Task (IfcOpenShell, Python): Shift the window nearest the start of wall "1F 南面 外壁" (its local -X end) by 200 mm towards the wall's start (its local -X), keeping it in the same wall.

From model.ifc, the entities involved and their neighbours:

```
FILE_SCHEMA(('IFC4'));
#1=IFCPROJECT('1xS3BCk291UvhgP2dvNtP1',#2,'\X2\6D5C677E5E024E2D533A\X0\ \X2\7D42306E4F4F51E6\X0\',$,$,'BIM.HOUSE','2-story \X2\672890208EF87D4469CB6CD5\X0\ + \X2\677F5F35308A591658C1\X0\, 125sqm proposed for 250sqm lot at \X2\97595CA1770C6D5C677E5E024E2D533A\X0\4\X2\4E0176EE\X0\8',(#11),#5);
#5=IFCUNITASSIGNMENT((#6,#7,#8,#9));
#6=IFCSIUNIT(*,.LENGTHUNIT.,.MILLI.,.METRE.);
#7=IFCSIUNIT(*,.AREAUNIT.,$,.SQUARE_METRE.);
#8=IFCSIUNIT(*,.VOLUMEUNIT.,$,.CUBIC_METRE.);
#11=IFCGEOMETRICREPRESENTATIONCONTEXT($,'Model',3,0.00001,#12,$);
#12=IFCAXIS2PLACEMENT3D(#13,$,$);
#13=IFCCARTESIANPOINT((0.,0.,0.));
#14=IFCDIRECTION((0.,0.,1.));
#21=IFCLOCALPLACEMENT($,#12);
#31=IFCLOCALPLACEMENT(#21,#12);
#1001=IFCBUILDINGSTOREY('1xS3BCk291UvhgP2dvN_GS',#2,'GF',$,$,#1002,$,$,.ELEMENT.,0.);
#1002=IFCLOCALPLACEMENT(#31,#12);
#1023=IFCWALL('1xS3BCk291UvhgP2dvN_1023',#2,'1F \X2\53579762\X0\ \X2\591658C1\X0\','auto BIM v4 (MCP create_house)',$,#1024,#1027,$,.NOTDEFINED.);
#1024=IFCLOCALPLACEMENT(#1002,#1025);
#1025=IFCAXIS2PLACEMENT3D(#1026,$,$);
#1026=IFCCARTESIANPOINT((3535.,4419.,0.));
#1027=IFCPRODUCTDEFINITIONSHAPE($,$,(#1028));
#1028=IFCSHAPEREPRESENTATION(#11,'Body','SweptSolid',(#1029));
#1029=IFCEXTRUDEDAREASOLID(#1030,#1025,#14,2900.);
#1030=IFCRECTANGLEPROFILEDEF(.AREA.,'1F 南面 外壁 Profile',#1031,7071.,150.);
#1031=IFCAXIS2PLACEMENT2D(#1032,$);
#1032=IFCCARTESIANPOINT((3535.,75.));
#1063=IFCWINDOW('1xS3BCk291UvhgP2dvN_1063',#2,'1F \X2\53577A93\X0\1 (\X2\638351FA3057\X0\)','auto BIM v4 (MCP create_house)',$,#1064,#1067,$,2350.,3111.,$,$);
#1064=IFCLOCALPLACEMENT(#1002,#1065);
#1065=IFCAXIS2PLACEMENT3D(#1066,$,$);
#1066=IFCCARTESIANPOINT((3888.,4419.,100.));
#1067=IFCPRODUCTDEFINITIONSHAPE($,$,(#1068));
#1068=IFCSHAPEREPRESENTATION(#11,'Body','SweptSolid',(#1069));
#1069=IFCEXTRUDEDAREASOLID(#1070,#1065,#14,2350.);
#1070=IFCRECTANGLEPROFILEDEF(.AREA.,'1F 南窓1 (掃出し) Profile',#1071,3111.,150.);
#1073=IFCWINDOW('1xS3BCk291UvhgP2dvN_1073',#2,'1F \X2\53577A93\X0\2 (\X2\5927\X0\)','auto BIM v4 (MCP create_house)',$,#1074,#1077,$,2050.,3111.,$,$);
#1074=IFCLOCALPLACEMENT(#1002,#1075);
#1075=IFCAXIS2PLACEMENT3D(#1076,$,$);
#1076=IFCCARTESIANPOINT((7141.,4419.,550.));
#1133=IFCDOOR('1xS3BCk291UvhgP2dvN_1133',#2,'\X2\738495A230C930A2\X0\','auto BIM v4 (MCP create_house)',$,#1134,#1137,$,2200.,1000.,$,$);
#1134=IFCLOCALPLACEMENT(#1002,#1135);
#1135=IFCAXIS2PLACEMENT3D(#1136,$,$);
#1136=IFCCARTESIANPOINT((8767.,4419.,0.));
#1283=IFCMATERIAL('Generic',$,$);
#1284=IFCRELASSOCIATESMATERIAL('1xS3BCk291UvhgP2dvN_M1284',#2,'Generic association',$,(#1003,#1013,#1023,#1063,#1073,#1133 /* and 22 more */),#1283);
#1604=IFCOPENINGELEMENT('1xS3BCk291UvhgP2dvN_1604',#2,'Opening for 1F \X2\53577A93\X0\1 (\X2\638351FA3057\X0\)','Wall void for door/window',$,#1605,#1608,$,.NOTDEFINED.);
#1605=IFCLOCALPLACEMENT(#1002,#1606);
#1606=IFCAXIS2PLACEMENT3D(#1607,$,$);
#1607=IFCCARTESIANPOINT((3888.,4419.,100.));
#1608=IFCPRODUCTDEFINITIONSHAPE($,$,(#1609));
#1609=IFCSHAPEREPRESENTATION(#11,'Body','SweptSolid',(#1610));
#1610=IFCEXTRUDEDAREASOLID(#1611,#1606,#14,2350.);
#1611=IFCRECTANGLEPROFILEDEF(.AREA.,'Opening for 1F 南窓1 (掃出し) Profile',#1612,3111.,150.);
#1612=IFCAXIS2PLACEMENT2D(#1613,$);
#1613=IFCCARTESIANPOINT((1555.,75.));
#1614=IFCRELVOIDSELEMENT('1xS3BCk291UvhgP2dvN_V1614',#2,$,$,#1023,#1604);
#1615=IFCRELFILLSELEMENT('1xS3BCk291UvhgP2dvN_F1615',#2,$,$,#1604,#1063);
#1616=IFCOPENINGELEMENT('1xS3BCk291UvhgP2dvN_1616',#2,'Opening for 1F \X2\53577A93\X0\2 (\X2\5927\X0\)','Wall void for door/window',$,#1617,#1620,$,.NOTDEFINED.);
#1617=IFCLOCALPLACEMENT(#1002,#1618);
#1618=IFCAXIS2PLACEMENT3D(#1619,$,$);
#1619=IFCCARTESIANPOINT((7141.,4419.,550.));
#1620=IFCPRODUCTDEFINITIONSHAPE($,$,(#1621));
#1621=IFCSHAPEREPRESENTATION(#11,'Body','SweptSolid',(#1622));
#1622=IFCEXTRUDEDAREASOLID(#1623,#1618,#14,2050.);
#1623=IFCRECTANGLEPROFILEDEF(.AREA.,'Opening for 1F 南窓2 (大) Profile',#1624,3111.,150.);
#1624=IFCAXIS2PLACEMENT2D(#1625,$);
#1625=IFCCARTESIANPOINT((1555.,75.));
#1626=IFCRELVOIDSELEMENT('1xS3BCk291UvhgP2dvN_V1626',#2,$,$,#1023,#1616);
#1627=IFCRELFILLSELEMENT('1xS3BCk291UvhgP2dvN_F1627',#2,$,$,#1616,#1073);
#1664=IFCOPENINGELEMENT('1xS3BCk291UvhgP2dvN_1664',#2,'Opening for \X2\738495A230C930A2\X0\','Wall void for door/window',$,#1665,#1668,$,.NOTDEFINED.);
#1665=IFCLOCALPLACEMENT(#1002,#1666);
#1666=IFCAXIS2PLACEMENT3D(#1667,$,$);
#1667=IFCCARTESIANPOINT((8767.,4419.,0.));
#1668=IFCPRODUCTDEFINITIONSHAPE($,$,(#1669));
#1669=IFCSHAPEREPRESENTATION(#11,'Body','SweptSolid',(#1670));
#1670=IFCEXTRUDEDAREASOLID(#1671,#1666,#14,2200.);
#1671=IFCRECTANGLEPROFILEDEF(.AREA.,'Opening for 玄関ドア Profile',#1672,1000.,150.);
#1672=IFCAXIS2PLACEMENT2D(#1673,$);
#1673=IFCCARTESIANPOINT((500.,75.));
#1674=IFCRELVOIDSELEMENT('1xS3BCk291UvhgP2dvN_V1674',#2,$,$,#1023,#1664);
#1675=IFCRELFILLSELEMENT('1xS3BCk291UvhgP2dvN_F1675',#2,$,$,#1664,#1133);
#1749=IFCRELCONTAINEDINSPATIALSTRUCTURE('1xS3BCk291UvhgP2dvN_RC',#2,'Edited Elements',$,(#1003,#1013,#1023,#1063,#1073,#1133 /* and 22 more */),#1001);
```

```python
import ifcopenshell
import ifcopenshell.api.geometry
import ifcopenshell.util.placement

model = ifcopenshell.open("model.ifc")

window = model.by_id(1063)
opening = window.FillsVoids[0].RelatingOpeningElement
wall = opening.VoidsElements[0].RelatingBuildingElement

wall_matrix = ifcopenshell.util.placement.get_local_placement(wall.ObjectPlacement)
shift = wall_matrix[:3, 0] * -200.0
before = ifcopenshell.util.placement.get_local_placement(window.ObjectPlacement)[:3, 3].copy()

# The window is not placed relative to its opening, so move both.
for product in (opening, window):
    matrix = ifcopenshell.util.placement.get_local_placement(product.ObjectPlacement)
    matrix[:3, 3] += shift
    ifcopenshell.api.geometry.edit_object_placement(model, product=product, matrix=matrix, is_si=False)

after = ifcopenshell.util.placement.get_local_placement(window.ObjectPlacement)[:3, 3]
print("window moved by", (after - before).round(3) + 0.0)

model.write("model_edited.ifc")
```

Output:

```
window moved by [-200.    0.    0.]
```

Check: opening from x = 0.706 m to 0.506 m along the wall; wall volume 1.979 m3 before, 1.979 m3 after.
